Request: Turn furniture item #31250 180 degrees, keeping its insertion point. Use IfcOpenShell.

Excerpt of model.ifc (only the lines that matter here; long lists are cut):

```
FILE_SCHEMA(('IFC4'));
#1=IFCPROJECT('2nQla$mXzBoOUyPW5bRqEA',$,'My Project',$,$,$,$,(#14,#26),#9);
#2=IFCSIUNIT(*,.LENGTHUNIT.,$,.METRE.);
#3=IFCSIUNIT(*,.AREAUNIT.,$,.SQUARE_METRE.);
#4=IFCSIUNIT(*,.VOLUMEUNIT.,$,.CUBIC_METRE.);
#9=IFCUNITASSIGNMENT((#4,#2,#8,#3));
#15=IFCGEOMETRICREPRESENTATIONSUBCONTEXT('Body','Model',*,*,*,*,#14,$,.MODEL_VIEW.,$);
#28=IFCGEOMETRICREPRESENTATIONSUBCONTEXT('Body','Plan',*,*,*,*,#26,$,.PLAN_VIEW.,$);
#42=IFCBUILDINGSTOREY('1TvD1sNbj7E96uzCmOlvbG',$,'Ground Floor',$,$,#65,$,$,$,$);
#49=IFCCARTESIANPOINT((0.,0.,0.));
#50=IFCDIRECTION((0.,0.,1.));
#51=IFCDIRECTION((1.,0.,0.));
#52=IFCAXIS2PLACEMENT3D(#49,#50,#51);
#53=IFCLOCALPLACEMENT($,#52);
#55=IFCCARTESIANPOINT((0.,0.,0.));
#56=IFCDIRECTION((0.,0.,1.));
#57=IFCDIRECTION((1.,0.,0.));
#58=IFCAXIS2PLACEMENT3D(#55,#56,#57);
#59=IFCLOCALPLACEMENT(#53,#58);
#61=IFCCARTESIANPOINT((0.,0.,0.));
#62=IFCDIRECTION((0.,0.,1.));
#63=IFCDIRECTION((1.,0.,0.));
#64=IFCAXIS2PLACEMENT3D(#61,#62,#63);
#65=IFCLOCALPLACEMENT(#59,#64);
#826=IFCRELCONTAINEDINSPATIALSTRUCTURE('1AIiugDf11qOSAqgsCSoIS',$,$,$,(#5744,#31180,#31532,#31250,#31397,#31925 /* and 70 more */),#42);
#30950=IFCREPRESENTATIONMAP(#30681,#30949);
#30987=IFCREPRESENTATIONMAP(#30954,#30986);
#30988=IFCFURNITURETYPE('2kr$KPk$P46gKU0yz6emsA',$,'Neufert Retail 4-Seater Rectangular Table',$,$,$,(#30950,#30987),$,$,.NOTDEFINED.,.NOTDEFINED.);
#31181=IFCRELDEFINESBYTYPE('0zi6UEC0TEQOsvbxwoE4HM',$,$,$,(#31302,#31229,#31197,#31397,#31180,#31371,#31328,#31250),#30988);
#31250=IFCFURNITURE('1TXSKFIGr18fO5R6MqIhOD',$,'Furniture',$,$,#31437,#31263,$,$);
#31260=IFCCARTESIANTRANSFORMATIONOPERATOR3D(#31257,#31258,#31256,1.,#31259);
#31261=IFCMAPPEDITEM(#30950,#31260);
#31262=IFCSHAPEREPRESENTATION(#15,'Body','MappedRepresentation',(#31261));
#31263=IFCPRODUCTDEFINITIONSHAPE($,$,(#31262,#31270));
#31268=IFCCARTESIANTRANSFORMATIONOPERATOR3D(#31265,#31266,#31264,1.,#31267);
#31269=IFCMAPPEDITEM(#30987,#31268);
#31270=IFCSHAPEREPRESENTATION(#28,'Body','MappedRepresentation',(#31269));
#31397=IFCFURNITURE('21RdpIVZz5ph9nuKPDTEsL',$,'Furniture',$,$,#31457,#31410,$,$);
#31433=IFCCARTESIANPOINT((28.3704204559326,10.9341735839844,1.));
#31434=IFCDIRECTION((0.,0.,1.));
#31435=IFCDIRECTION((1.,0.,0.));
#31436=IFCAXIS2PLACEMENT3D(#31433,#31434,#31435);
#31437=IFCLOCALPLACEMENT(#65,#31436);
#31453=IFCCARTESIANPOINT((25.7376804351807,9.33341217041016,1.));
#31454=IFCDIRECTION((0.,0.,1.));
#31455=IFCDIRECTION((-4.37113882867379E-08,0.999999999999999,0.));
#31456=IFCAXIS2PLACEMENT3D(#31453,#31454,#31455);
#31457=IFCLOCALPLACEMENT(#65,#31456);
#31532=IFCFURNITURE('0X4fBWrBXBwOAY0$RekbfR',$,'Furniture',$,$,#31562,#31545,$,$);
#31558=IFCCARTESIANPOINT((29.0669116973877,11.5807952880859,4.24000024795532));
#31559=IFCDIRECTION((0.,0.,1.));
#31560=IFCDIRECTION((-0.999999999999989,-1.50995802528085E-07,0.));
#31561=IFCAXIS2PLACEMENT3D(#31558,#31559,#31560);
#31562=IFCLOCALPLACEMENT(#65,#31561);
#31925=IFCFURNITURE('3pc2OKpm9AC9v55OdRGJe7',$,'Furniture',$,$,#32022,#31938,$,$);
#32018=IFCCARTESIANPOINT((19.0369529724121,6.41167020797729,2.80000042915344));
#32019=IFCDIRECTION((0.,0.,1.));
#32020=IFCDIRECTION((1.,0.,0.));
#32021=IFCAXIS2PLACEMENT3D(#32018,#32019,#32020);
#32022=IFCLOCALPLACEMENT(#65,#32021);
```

```python
import ifcopenshell
import ifcopenshell.api.geometry
import ifcopenshell.util.placement

model = ifcopenshell.open("model.ifc")

item = model.by_guid("1TXSKFIGr18fO5R6MqIhOD")
matrix = ifcopenshell.util.placement.get_local_placement(item.ObjectPlacement)
matrix = matrix @ ifcopenshell.util.placement.rotation(180, "Z")
ifcopenshell.api.geometry.edit_object_placement(model, product=item, matrix=matrix, is_si=False)

print(ifcopenshell.util.placement.get_local_placement(item.ObjectPlacement).round(3) + 0.0)

model.write("model_v2.ifc")
```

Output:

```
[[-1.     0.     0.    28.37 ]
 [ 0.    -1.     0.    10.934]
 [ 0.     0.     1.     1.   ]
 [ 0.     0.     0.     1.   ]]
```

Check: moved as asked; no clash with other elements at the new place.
